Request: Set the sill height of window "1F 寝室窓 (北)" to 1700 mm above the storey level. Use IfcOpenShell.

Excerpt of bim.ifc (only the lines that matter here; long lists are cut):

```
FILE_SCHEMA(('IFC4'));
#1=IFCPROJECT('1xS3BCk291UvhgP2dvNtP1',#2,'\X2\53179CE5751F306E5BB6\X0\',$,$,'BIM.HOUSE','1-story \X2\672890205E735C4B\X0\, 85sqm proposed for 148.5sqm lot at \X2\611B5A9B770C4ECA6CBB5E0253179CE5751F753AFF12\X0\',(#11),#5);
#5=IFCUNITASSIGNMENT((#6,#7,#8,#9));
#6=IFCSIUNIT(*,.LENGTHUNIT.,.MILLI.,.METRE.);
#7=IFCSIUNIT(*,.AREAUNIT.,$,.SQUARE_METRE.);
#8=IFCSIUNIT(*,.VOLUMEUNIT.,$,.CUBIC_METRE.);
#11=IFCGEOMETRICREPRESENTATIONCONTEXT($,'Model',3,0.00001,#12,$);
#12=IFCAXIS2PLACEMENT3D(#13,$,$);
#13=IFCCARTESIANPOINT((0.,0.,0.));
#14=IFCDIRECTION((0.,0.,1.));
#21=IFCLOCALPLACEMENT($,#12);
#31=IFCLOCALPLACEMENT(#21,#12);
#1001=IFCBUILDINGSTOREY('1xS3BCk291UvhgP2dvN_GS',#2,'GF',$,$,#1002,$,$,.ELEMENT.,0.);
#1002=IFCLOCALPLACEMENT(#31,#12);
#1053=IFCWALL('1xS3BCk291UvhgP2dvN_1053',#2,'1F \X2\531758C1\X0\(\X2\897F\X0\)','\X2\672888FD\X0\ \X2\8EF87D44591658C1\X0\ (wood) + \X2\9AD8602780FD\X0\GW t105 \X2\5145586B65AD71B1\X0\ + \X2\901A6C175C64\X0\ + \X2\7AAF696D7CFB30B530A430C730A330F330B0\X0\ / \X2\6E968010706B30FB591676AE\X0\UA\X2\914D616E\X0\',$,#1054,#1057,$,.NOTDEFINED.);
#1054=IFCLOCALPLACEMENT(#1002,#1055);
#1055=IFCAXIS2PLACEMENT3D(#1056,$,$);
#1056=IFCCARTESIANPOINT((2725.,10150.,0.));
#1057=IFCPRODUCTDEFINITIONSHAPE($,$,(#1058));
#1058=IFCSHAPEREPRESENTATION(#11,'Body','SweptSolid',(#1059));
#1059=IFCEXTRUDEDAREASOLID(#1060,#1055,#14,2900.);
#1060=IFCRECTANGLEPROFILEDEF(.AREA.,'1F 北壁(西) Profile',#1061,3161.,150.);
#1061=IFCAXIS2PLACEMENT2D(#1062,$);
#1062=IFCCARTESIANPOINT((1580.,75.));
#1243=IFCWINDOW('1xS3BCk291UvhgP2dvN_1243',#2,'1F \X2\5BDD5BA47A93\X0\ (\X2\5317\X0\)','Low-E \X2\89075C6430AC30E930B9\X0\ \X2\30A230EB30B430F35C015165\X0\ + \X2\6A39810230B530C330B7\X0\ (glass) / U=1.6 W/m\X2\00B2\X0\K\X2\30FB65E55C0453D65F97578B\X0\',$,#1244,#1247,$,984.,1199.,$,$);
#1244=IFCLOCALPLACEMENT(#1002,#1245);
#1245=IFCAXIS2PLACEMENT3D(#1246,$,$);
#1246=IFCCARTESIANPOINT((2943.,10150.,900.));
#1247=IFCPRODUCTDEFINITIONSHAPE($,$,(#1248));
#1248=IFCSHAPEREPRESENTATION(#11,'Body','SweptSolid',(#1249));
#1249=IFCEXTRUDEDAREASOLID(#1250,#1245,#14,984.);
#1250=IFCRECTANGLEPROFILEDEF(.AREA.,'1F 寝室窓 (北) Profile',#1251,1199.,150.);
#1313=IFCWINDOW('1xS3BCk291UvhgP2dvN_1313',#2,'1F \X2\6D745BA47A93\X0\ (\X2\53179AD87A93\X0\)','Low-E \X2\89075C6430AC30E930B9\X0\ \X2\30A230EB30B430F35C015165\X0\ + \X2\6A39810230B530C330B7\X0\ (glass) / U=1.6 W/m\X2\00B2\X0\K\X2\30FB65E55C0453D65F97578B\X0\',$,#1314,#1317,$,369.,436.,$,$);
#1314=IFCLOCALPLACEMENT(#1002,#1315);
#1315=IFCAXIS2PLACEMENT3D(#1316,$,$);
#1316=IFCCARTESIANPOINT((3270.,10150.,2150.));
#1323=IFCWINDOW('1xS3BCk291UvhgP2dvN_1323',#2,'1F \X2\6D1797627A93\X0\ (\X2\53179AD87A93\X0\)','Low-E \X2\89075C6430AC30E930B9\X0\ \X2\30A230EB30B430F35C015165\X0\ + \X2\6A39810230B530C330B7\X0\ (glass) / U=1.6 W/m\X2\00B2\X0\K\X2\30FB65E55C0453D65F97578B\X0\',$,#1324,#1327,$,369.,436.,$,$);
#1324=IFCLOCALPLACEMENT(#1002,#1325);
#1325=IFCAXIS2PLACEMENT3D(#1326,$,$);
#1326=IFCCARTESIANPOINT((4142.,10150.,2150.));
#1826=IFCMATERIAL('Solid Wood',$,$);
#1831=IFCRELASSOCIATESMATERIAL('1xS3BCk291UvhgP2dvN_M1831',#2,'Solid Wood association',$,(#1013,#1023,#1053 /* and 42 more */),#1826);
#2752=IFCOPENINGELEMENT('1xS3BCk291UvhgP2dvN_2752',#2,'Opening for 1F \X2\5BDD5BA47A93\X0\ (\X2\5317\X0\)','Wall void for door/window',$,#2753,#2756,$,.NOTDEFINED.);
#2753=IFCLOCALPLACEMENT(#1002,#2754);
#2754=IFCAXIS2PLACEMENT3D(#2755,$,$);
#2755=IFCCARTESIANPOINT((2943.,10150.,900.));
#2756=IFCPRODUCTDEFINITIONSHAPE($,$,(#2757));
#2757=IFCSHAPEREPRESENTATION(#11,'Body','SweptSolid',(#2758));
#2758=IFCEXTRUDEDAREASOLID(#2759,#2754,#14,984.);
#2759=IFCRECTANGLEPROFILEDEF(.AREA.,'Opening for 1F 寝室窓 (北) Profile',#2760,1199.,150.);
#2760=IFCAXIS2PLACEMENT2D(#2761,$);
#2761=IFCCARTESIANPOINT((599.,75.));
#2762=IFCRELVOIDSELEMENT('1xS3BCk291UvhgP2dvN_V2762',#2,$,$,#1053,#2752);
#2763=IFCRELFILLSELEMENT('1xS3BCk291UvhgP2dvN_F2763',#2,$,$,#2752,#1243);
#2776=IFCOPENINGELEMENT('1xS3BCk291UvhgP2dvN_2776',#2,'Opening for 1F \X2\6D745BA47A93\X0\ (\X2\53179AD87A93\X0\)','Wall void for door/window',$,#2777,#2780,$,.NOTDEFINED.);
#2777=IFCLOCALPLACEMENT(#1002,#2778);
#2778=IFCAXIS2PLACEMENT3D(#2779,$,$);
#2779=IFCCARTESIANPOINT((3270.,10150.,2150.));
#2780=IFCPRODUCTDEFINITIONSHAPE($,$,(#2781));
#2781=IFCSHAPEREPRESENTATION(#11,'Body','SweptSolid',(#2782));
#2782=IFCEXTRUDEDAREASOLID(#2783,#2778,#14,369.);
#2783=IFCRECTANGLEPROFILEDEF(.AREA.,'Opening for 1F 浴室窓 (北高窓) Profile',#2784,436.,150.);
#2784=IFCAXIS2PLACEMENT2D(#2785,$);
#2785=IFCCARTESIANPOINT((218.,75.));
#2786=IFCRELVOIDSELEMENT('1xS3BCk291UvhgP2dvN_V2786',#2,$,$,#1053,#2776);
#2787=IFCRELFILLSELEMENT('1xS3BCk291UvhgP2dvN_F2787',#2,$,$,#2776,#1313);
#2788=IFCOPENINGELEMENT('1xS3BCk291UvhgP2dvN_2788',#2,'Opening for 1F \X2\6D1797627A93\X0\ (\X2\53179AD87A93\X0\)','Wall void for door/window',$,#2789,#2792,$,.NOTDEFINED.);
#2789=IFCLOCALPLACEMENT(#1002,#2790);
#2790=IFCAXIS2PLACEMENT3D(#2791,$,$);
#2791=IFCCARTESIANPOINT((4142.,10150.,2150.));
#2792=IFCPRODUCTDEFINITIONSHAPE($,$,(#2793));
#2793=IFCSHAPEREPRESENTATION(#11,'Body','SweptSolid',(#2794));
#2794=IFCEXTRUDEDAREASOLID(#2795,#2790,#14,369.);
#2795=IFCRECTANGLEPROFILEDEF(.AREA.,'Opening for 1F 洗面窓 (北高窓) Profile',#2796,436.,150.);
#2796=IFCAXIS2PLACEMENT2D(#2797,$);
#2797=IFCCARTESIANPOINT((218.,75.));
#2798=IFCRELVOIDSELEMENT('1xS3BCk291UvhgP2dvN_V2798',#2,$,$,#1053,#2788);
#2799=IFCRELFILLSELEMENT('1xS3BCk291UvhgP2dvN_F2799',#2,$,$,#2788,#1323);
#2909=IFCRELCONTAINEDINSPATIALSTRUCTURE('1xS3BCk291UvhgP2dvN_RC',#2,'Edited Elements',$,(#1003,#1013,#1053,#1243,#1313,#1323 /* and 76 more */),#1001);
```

```python
import numpy as np
import ifcopenshell
import ifcopenshell.api.geometry
import ifcopenshell.geom
import ifcopenshell.util.element
import ifcopenshell.util.placement
import ifcopenshell.util.shape
import ifcopenshell.util.unit

model = ifcopenshell.open("bim.ifc")
unit_scale = ifcopenshell.util.unit.calculate_unit_scale(model)

window = model.by_guid("1xS3BCk291UvhgP2dvN_1243")
opening = window.FillsVoids[0].RelatingOpeningElement
storey = ifcopenshell.util.element.get_container(window, ifc_class="IfcBuildingStorey")
level = ifcopenshell.util.placement.get_local_placement(storey.ObjectPlacement)[2, 3]

# The opening's origin need not be at the sill, so measure its lowest point.
shape = ifcopenshell.geom.create_shape(ifcopenshell.geom.settings(), opening)
bottom = ifcopenshell.util.shape.get_shape_bottom_elevation(shape, shape.geometry) / unit_scale
dz = level + 1.7 / unit_scale - bottom

shift = np.array([0.0, 0.0, dz])
# The window is not placed relative to its opening, so move both.
for product in (opening, window):
    matrix = ifcopenshell.util.placement.get_local_placement(product.ObjectPlacement)
    matrix[:3, 3] += shift
    ifcopenshell.api.geometry.edit_object_placement(model, product=product, matrix=matrix, is_si=False)

print(f"moved by {dz * unit_scale:+.3f} m")

model.write("bim_updated.ifc")
```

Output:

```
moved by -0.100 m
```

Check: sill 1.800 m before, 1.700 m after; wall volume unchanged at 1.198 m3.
